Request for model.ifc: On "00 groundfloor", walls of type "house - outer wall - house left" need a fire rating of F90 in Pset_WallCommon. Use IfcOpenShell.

First a look at what the model holds.

```python
import ifcopenshell
import ifcopenshell.util.element

model = ifcopenshell.open("model.ifc")
print(model.schema)
storey = next(s for s in model.by_type("IfcBuildingStorey") if s.Name == "00 groundfloor")
walls = [e for e in ifcopenshell.util.element.get_decomposition(storey) if e.is_a("IfcWall")]
seen = {}
for e in walls:
    element_type = ifcopenshell.util.element.get_type(e)
    key = (element_type.Name if element_type != e and element_type else None, ifcopenshell.util.element.get_pset(e, "Pset_WallCommon", "FireRating"))
    seen[key] = seen.get(key, 0) + 1
for (name, value), count in sorted(seen.items(), key=str):
    print(count, "x", name, "|", value)
```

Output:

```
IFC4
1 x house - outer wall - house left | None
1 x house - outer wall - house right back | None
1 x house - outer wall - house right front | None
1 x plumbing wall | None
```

```python
import ifcopenshell
import ifcopenshell.api.pset
import ifcopenshell.util.element

model = ifcopenshell.open("model.ifc")

storey = next(s for s in model.by_type("IfcBuildingStorey") if s.Name == "00 groundfloor")
walls = [e for e in ifcopenshell.util.element.get_decomposition(storey) if e.is_a("IfcWall")]

count = 0
for e in walls:
    element_type = ifcopenshell.util.element.get_type(e)
    if element_type in (None, e) or element_type.Name != "house - outer wall - house left":
        continue
    # add_pset returns the element's existing set when there is one.
    pset = ifcopenshell.api.pset.add_pset(model, product=e, name="Pset_WallCommon")
    ifcopenshell.api.pset.edit_pset(model, pset=pset, properties={"FireRating": "F90"})
    count += 1

print(count, "walls updated")

model.write("model_rev.ifc")
```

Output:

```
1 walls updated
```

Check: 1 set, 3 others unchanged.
